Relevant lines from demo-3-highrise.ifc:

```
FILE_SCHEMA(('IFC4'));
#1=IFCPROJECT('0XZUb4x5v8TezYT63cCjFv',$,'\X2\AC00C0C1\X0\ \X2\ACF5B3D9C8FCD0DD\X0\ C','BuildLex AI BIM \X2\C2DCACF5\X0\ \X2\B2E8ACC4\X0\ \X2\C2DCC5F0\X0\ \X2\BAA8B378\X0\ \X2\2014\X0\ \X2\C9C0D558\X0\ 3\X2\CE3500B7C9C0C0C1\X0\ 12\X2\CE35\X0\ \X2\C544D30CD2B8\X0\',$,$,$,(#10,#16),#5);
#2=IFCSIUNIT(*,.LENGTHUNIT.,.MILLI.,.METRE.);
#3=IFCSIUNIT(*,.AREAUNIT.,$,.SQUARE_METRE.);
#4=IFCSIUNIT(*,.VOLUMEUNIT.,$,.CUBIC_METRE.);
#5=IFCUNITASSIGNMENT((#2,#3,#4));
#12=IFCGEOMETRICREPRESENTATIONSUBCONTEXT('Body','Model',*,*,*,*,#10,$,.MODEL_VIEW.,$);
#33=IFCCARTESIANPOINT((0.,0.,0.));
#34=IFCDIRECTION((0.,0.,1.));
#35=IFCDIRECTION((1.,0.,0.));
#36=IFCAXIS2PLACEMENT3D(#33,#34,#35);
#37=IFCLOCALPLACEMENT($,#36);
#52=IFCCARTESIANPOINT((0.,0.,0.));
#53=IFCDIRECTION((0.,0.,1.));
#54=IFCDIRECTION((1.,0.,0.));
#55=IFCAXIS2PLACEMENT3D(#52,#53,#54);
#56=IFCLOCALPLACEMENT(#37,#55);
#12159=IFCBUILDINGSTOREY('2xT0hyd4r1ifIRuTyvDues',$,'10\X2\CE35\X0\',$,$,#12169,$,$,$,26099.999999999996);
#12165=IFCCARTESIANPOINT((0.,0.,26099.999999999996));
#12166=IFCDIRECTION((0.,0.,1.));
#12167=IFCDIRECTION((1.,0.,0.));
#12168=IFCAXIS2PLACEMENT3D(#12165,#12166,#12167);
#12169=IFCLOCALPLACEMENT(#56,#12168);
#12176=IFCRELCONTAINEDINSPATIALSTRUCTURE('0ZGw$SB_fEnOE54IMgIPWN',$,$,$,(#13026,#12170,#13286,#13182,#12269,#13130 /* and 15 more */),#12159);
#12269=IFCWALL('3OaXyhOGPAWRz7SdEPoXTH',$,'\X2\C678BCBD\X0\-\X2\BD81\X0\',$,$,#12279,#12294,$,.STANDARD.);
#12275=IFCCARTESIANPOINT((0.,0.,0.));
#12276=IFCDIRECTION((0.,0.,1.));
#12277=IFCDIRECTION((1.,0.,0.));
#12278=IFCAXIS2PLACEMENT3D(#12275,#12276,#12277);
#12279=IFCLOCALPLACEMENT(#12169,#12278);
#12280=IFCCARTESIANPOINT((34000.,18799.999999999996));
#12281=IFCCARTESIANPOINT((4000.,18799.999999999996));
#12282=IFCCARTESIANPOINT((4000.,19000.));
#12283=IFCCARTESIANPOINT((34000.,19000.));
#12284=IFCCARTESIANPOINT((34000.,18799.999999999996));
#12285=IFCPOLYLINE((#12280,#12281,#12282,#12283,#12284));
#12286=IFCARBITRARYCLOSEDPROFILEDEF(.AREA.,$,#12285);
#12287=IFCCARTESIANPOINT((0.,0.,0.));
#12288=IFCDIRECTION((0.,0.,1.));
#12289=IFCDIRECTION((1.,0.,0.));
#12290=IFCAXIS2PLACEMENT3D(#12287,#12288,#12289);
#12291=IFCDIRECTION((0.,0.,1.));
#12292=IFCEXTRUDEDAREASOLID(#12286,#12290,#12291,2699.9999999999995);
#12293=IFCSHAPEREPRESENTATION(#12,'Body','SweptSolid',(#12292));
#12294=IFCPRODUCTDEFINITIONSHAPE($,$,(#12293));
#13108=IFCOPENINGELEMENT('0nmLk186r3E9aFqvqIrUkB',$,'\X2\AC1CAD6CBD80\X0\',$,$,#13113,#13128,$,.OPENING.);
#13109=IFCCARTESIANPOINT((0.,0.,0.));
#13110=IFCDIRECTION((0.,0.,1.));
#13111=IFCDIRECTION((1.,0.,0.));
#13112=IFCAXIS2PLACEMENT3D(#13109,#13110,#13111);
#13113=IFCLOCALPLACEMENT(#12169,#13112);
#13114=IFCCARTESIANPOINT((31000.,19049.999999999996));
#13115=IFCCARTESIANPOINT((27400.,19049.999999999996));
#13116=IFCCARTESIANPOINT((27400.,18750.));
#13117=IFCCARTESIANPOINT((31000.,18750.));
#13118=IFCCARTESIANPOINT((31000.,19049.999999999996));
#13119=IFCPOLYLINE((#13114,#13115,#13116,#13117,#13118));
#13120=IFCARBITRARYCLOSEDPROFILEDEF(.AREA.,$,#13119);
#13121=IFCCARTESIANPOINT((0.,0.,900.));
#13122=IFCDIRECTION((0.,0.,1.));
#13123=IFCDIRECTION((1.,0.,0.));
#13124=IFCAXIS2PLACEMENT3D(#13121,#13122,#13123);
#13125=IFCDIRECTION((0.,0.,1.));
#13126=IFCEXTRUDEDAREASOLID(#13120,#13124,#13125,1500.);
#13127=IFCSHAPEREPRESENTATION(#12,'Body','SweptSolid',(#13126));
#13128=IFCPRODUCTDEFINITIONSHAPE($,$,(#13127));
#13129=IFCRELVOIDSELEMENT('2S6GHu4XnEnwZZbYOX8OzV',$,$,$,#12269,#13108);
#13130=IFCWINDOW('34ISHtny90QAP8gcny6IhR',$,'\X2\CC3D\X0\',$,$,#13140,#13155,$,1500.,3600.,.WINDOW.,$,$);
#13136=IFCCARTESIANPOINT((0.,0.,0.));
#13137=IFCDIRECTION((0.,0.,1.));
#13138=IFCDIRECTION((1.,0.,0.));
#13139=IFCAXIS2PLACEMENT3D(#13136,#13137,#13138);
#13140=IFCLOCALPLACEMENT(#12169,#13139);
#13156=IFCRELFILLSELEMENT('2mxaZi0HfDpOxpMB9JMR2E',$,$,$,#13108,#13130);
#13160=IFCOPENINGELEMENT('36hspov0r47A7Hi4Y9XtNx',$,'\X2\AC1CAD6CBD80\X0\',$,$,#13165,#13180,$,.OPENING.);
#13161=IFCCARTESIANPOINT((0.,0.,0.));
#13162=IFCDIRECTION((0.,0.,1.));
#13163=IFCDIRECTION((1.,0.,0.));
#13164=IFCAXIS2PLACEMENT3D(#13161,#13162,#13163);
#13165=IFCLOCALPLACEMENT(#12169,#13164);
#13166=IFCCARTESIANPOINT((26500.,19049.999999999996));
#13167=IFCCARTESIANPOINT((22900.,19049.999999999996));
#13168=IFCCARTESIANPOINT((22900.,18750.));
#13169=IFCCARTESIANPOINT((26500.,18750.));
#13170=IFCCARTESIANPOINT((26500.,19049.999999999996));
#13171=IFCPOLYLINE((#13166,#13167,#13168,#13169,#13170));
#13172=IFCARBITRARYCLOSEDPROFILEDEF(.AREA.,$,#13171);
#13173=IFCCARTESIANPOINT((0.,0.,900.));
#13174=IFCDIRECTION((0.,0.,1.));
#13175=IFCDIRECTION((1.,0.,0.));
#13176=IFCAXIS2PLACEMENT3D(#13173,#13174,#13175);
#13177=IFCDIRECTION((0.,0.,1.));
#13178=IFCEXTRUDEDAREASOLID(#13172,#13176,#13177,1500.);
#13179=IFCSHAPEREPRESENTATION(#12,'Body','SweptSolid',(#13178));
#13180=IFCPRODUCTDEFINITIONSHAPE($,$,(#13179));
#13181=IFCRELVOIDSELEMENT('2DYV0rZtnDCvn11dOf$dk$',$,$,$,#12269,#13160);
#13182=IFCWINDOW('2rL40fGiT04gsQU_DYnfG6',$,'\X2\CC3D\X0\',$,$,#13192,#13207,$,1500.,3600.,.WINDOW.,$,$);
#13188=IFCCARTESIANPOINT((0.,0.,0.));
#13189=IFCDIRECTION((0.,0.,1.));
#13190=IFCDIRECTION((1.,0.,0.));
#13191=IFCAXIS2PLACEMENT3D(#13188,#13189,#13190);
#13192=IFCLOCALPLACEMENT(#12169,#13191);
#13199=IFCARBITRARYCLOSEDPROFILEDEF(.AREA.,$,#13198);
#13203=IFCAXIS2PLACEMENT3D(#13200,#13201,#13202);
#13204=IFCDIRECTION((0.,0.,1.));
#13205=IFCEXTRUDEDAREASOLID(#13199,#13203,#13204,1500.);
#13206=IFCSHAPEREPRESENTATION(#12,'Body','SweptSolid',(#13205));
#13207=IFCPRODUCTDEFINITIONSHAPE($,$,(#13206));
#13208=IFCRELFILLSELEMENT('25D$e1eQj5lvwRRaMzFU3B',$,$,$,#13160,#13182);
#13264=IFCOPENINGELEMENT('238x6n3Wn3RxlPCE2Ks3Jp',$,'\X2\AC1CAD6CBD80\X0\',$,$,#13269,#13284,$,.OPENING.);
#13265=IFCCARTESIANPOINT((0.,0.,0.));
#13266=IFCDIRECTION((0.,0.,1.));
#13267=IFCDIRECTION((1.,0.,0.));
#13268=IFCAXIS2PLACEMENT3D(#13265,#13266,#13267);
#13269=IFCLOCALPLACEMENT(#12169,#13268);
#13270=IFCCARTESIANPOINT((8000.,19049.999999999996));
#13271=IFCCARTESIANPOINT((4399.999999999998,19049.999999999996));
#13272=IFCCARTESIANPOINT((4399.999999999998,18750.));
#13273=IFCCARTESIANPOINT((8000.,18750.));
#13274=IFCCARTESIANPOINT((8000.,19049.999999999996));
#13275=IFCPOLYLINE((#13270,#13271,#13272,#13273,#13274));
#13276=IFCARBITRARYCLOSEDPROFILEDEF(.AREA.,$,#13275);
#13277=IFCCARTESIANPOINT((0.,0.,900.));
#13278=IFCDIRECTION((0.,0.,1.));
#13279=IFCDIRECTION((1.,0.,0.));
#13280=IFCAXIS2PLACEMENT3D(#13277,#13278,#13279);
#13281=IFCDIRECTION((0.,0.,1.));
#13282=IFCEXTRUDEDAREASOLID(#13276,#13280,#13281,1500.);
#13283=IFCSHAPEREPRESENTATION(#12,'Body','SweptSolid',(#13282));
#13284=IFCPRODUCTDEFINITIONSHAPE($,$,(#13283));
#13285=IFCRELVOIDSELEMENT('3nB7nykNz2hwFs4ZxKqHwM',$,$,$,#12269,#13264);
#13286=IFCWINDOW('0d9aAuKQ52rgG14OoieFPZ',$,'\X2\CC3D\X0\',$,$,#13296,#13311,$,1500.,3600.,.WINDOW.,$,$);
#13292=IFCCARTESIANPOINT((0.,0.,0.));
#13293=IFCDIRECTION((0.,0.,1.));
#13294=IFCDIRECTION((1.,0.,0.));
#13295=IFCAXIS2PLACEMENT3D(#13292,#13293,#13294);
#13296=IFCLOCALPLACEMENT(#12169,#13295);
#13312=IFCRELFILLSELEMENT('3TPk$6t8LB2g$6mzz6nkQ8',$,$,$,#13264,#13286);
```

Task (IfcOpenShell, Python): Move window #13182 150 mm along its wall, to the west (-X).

```python
import ifcopenshell
import ifcopenshell.api.geometry
import ifcopenshell.util.placement

model = ifcopenshell.open("demo-3-highrise.ifc")

window = model.by_id(13182)
opening = window.FillsVoids[0].RelatingOpeningElement
wall = opening.VoidsElements[0].RelatingBuildingElement

wall_matrix = ifcopenshell.util.placement.get_local_placement(wall.ObjectPlacement)
shift = wall_matrix[:3, 0] * -150.0
before = ifcopenshell.util.placement.get_local_placement(window.ObjectPlacement)[:3, 3].copy()

# The window is not placed relative to its opening, so move both.
for product in (opening, window):
    matrix = ifcopenshell.util.placement.get_local_placement(product.ObjectPlacement)
    matrix[:3, 3] += shift
    ifcopenshell.api.geometry.edit_object_placement(model, product=product, matrix=matrix, is_si=False)

after = ifcopenshell.util.placement.get_local_placement(window.ObjectPlacement)[:3, 3]
print("window moved by", (after - before).round(3) + 0.0)

model.write("demo-3-highrise_updated.ifc")
```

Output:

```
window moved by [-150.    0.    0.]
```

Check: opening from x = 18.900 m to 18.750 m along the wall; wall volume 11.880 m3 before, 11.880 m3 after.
